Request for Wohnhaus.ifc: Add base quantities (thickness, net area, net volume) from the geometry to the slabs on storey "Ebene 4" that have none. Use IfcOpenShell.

First a look at what the model holds.

```python
import ifcopenshell
import ifcopenshell.util.element
import ifcopenshell.util.unit

model = ifcopenshell.open("Wohnhaus.ifc")
print(model.schema)
for unit_type in ("LENGTHUNIT", "AREAUNIT", "VOLUMEUNIT"):
    print(unit_type, ifcopenshell.util.unit.calculate_unit_scale(model, unit_type))
storey = next(s for s in model.by_type("IfcBuildingStorey") if s.Name == "Ebene 4")
slabs = [e for e in ifcopenshell.util.element.get_decomposition(storey) if e.is_a("IfcSlab")]
for e in sorted(slabs, key=lambda e: e.id()):
    print(e.id(), e.is_a(), e.Name, list(ifcopenshell.util.element.get_psets(e, qtos_only=True)), sep=" | ")
```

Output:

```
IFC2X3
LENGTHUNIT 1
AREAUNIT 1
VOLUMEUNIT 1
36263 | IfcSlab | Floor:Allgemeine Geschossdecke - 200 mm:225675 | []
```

```python
import ifcopenshell
import ifcopenshell.api.pset
import ifcopenshell.geom
import ifcopenshell.util.element
import ifcopenshell.util.shape
import ifcopenshell.util.unit

model = ifcopenshell.open("Wohnhaus.ifc")
unit_scale = ifcopenshell.util.unit.calculate_unit_scale(model)
area_scale = ifcopenshell.util.unit.calculate_unit_scale(model, "AREAUNIT")
volume_scale = ifcopenshell.util.unit.calculate_unit_scale(model, "VOLUMEUNIT")
settings = ifcopenshell.geom.settings()

storey = next(s for s in model.by_type("IfcBuildingStorey") if s.Name == "Ebene 4")
slabs = [e for e in ifcopenshell.util.element.get_decomposition(storey) if e.is_a("IfcSlab")]

for e in sorted(slabs, key=lambda e: e.id()):
    if ifcopenshell.util.element.get_psets(e, qtos_only=True, should_inherit=False):
        continue
    # Geometry comes back in metres, in the element's own axes.
    shape = ifcopenshell.geom.create_shape(settings, e)
    values = {
        "Width": ifcopenshell.util.shape.get_z(shape.geometry) / unit_scale,
        "NetArea": ifcopenshell.util.shape.get_footprint_area(shape.geometry) / area_scale,
        "NetVolume": ifcopenshell.util.shape.get_volume(shape.geometry) / volume_scale,
    }
    qto = ifcopenshell.api.pset.add_qto(model, product=e, name="BaseQuantities")
    ifcopenshell.api.pset.edit_qto(model, qto=qto, properties=values)
    print(e.id(), {k: round(v, 3) for k, v in values.items()})

model.write("Wohnhaus-out.ifc")
```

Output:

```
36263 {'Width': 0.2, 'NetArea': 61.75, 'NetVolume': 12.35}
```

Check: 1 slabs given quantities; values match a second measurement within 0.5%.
